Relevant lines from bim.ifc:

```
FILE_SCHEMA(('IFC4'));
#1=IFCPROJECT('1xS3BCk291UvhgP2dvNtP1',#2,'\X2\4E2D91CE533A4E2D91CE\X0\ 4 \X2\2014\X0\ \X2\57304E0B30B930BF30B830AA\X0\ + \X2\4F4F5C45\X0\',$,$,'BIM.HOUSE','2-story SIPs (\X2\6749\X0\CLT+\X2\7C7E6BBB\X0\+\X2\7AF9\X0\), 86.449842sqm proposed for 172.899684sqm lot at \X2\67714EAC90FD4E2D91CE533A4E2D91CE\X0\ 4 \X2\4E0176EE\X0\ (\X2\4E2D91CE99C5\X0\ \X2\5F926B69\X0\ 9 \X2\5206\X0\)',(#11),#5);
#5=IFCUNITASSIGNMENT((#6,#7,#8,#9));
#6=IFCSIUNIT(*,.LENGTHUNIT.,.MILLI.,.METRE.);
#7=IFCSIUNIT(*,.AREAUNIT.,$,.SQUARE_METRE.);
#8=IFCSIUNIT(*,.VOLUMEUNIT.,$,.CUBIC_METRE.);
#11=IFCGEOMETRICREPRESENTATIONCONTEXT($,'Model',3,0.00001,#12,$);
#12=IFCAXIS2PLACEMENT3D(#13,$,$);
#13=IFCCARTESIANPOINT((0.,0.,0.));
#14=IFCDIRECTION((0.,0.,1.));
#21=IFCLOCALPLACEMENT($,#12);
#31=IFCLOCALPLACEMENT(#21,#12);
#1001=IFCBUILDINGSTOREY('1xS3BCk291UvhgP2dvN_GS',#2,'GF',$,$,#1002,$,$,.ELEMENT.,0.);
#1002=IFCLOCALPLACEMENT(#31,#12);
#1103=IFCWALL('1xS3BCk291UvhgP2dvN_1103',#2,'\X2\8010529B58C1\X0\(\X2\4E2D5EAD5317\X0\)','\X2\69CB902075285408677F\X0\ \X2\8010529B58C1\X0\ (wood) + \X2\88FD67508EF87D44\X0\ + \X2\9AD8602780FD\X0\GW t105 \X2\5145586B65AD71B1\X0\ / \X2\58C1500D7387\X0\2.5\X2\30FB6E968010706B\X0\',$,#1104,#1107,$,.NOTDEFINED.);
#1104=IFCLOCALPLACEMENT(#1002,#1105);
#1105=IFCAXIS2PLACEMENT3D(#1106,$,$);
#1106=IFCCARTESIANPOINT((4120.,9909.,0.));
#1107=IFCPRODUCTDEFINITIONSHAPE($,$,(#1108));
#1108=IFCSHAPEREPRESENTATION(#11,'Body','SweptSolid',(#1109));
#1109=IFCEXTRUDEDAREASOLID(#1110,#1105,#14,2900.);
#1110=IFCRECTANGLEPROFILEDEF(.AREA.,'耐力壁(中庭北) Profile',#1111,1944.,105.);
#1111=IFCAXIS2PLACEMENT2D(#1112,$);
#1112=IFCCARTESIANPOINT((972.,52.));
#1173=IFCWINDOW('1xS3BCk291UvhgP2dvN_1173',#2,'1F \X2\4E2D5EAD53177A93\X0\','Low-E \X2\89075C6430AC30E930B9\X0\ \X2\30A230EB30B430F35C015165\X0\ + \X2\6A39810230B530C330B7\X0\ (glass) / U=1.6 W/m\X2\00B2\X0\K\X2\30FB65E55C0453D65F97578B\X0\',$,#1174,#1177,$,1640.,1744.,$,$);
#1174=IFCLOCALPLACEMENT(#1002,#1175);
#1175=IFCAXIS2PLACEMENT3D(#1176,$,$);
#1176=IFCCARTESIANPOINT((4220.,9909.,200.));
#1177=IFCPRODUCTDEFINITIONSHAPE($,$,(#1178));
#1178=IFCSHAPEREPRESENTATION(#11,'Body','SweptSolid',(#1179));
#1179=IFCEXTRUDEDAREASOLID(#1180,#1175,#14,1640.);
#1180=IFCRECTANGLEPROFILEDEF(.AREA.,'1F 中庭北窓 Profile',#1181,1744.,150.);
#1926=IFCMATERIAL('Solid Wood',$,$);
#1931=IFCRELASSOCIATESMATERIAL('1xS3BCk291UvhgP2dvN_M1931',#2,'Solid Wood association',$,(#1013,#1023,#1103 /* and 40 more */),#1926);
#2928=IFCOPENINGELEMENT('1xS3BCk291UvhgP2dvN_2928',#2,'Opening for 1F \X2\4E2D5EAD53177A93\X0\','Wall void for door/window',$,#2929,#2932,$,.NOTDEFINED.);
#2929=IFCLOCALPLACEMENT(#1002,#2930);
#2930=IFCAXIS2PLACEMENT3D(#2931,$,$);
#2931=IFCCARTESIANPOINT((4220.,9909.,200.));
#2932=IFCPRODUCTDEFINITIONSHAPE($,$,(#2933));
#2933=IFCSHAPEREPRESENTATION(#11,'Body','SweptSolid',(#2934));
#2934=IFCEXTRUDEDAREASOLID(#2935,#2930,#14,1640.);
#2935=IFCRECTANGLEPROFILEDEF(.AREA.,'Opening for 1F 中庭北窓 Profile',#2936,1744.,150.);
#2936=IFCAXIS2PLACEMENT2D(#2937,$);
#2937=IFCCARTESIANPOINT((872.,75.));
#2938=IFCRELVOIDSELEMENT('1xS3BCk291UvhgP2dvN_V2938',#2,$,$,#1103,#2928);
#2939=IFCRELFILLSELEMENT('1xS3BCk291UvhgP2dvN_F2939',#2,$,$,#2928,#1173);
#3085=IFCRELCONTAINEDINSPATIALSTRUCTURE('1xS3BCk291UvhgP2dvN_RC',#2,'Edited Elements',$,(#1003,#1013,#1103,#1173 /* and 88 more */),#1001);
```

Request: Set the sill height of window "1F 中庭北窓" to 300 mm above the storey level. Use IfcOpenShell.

```python
import numpy as np
import ifcopenshell
import ifcopenshell.api.geometry
import ifcopenshell.geom
import ifcopenshell.util.element
import ifcopenshell.util.placement
import ifcopenshell.util.shape
import ifcopenshell.util.unit

model = ifcopenshell.open("bim.ifc")
unit_scale = ifcopenshell.util.unit.calculate_unit_scale(model)

window = model.by_guid("1xS3BCk291UvhgP2dvN_1173")
opening = window.FillsVoids[0].RelatingOpeningElement
storey = ifcopenshell.util.element.get_container(window, ifc_class="IfcBuildingStorey")
level = ifcopenshell.util.placement.get_local_placement(storey.ObjectPlacement)[2, 3]

# The opening's origin need not be at the sill, so measure its lowest point.
shape = ifcopenshell.geom.create_shape(ifcopenshell.geom.settings(), opening)
bottom = ifcopenshell.util.shape.get_shape_bottom_elevation(shape, shape.geometry) / unit_scale
dz = level + 0.3 / unit_scale - bottom

shift = np.array([0.0, 0.0, dz])
# The window is not placed relative to its opening, so move both.
for product in (opening, window):
    matrix = ifcopenshell.util.placement.get_local_placement(product.ObjectPlacement)
    matrix[:3, 3] += shift
    ifcopenshell.api.geometry.edit_object_placement(model, product=product, matrix=matrix, is_si=False)

print(f"moved by {dz * unit_scale:+.3f} m")

model.write("bim_v2.ifc")
```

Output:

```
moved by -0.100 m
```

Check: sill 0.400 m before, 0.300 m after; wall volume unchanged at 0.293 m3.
